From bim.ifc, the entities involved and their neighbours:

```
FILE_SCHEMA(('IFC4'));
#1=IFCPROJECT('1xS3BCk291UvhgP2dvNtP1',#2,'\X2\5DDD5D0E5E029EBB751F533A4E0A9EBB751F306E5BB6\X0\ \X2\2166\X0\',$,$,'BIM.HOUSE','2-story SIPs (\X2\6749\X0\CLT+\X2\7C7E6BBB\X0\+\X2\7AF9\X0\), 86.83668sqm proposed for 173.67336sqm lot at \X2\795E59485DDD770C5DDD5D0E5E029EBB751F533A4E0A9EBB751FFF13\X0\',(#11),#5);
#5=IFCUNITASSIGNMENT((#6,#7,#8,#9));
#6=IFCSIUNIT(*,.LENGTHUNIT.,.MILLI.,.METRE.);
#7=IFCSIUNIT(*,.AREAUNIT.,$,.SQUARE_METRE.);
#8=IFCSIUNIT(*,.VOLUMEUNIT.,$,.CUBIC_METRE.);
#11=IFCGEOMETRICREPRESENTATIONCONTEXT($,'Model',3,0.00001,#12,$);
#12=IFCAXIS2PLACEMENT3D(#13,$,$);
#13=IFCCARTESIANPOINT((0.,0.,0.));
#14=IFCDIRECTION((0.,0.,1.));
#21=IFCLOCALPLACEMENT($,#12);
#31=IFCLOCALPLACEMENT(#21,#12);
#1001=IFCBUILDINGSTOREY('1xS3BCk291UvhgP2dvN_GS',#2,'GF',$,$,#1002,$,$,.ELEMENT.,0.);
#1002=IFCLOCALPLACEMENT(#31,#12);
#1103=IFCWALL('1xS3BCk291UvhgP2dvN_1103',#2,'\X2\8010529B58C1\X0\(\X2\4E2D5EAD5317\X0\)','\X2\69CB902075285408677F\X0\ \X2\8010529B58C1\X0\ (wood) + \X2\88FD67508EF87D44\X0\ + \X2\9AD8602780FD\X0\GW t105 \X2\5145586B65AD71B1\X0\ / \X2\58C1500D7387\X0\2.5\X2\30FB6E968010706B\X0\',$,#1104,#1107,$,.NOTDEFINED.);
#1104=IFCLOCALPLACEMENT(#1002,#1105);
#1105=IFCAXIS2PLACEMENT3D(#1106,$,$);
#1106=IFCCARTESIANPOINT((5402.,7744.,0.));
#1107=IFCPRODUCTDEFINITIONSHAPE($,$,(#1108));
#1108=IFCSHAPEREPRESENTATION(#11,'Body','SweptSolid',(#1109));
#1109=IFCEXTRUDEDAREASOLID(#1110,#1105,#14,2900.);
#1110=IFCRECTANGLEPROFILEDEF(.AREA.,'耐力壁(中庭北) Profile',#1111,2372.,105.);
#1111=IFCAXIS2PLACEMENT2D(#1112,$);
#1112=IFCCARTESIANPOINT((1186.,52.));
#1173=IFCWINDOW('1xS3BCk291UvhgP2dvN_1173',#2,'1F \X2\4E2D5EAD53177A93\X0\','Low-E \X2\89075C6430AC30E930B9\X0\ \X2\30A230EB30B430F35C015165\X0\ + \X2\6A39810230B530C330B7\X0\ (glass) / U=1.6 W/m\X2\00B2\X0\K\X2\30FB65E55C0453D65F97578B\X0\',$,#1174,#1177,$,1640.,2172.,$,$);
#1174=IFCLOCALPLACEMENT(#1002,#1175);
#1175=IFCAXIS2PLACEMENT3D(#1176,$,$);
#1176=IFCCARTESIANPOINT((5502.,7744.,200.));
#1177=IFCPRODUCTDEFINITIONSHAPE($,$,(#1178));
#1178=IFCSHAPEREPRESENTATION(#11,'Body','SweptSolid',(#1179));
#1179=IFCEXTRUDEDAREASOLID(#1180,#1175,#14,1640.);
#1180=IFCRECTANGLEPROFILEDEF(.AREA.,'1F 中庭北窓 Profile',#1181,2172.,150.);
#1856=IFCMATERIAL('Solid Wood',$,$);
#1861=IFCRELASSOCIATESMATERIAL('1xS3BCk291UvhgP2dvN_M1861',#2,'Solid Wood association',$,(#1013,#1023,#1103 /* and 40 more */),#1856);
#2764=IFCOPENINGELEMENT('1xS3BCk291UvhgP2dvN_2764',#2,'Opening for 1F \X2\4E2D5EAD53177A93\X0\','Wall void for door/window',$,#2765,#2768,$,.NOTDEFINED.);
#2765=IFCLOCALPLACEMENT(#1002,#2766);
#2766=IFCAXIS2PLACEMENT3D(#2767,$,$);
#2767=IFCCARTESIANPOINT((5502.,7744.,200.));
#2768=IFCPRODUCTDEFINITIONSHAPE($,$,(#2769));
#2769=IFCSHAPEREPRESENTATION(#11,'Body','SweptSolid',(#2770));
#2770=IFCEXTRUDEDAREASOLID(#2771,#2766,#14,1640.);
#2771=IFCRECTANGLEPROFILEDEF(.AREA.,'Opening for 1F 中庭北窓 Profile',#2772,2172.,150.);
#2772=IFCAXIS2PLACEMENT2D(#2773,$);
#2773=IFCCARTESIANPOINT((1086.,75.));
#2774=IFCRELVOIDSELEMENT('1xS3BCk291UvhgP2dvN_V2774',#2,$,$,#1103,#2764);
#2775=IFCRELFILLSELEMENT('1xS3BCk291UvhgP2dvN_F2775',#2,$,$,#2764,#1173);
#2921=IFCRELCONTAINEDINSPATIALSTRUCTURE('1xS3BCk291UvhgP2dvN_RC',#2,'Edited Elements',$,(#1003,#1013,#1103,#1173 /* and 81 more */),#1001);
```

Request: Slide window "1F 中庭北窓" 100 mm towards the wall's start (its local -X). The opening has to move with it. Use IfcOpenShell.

```python
import ifcopenshell
import ifcopenshell.api.geometry
import ifcopenshell.util.placement
import ifcopenshell.util.unit

model = ifcopenshell.open("bim.ifc")
unit_scale = ifcopenshell.util.unit.calculate_unit_scale(model)

window = model.by_id(1173)
opening = window.FillsVoids[0].RelatingOpeningElement
wall = opening.VoidsElements[0].RelatingBuildingElement

wall_matrix = ifcopenshell.util.placement.get_local_placement(wall.ObjectPlacement)
shift = wall_matrix[:3, 0] * -0.1 / unit_scale
before = ifcopenshell.util.placement.get_local_placement(window.ObjectPlacement)[:3, 3].copy()

# The window is not placed relative to its opening, so move both.
for product in (opening, window):
    matrix = ifcopenshell.util.placement.get_local_placement(product.ObjectPlacement)
    matrix[:3, 3] += shift
    ifcopenshell.api.geometry.edit_object_placement(model, product=product, matrix=matrix, is_si=False)

after = ifcopenshell.util.placement.get_local_placement(window.ObjectPlacement)[:3, 3]
print("window moved by", (after - before).round(3) + 0.0)

model.write("bim_updated.ifc")
```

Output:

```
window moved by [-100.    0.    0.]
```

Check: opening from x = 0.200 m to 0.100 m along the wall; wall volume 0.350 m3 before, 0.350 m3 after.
